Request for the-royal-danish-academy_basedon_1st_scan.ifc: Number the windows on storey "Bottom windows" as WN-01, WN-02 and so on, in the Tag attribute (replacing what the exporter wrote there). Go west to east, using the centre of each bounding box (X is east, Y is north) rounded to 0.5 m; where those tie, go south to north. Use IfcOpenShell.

First a look at what the model holds.

```python
import ifcopenshell
import ifcopenshell.util.element
import ifcopenshell.util.placement

model = ifcopenshell.open("the-royal-danish-academy_basedon_1st_scan.ifc")
print(model.schema)
storey = next(s for s in model.by_type("IfcBuildingStorey") if s.Name == "Bottom windows")
windows = [e for e in ifcopenshell.util.element.get_decomposition(storey) if e.is_a("IfcWindow")]
for e in sorted(windows, key=lambda e: e.id()):
    origin = ifcopenshell.util.placement.get_local_placement(e.ObjectPlacement)[:3, 3]
    print(e.id(), e.Tag, e.Name, origin.round(2) + 0.0, sep=" | ")
```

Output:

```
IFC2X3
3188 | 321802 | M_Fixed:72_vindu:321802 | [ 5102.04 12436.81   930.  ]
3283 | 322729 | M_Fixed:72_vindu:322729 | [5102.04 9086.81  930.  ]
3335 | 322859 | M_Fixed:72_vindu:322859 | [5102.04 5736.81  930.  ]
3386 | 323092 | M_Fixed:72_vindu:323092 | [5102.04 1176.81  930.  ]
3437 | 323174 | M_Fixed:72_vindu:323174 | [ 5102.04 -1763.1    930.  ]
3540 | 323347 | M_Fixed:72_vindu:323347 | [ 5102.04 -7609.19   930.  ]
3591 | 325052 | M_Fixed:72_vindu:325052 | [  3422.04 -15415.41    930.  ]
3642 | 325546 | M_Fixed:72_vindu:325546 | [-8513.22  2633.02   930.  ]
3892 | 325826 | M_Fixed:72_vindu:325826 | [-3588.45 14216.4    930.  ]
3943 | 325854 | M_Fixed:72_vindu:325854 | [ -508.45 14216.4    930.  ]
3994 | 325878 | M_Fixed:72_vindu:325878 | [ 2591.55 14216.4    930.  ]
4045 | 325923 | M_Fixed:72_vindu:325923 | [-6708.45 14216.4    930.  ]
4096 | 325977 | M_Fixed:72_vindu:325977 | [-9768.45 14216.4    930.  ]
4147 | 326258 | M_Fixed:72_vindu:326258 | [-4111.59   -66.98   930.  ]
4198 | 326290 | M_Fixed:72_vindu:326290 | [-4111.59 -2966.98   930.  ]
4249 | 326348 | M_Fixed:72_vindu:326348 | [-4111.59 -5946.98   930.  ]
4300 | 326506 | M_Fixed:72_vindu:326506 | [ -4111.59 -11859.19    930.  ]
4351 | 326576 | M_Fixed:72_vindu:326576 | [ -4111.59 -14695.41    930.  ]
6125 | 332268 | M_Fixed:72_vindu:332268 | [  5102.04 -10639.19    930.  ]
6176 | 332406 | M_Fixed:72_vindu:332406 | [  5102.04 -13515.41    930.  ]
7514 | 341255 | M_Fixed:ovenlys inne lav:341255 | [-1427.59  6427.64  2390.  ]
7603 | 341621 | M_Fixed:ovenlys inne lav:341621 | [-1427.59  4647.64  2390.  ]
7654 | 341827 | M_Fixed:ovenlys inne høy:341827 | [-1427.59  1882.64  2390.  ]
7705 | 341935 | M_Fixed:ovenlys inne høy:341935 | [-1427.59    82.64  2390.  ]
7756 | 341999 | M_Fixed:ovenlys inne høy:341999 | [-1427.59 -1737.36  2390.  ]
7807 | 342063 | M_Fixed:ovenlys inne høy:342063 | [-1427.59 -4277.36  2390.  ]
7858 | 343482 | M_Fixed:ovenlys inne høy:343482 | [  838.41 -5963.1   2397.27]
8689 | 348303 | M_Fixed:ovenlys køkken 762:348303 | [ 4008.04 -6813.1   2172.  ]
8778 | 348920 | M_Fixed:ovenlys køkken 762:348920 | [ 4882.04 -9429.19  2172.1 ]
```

```python
import ifcopenshell
import ifcopenshell.geom
import ifcopenshell.util.element
import ifcopenshell.util.shape

model = ifcopenshell.open("the-royal-danish-academy_basedon_1st_scan.ifc")
settings = ifcopenshell.geom.settings()
settings.set("use-world-coords", True)


def centre(element):
    shape = ifcopenshell.geom.create_shape(settings, element)
    return ifcopenshell.util.shape.get_bbox_centroid(shape.geometry)


storey = next(s for s in model.by_type("IfcBuildingStorey") if s.Name == "Bottom windows")
windows = [e for e in ifcopenshell.util.element.get_decomposition(storey) if e.is_a("IfcWindow")]

# Insertion points can sit at a corner or the storey origin, so sort by the geometry (in metres).
centres = {e: centre(e) for e in windows}
windows.sort(key=lambda e: (round(centres[e][0] / 0.5), centres[e][1]))

for i, e in enumerate(windows, start=1):
    number = f"WN-{i:02d}"
    e.Tag = number
    print(e.id(), number)

model.write("the-royal-danish-academy_basedon_1st_scan_rev.ifc")
```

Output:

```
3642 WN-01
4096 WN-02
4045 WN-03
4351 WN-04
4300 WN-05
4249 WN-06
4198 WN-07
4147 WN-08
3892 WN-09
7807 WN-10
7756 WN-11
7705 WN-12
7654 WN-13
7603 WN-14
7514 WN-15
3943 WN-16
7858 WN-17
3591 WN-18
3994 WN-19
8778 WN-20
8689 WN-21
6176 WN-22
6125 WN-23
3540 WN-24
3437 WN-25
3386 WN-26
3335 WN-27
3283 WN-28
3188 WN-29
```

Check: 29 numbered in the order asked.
